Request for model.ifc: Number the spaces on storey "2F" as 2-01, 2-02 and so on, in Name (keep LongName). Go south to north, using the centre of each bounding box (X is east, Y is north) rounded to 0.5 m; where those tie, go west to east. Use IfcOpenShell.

First a look at what the model holds.

```python
import ifcopenshell
import ifcopenshell.util.element
import ifcopenshell.util.placement

model = ifcopenshell.open("model.ifc")
print(model.schema)
storey = next(s for s in model.by_type("IfcBuildingStorey") if s.Name == "2F")
spaces = [e for e in ifcopenshell.util.element.get_decomposition(storey) if e.is_a("IfcSpace")]
for e in sorted(spaces, key=lambda e: e.id()):
    origin = ifcopenshell.util.placement.get_local_placement(e.ObjectPlacement)[:3, 3]
    print(e.id(), e.Name, e.LongName, origin.round(2) + 0.0, sep=" | ")
```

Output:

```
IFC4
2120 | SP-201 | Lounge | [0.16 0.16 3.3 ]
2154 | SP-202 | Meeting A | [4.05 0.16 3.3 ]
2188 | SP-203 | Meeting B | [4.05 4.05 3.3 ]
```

```python
import ifcopenshell
import ifcopenshell.geom
import ifcopenshell.util.element
import ifcopenshell.util.shape

model = ifcopenshell.open("model.ifc")
settings = ifcopenshell.geom.settings()
settings.set("use-world-coords", True)


def centre(element):
    shape = ifcopenshell.geom.create_shape(settings, element)
    return ifcopenshell.util.shape.get_bbox_centroid(shape.geometry)


storey = next(s for s in model.by_type("IfcBuildingStorey") if s.Name == "2F")
spaces = [e for e in ifcopenshell.util.element.get_decomposition(storey) if e.is_a("IfcSpace")]

# Insertion points can sit at a corner or the storey origin, so sort by the geometry (in metres).
centres = {e: centre(e) for e in spaces}
spaces.sort(key=lambda e: (round(centres[e][1] / 0.5), centres[e][0]))

for i, e in enumerate(spaces, start=1):
    number = f"2-{i:02d}"
    e.Name = number
    print(e.id(), number)

model.write("model-out.ifc")
```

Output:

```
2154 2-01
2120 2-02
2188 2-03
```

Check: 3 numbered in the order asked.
